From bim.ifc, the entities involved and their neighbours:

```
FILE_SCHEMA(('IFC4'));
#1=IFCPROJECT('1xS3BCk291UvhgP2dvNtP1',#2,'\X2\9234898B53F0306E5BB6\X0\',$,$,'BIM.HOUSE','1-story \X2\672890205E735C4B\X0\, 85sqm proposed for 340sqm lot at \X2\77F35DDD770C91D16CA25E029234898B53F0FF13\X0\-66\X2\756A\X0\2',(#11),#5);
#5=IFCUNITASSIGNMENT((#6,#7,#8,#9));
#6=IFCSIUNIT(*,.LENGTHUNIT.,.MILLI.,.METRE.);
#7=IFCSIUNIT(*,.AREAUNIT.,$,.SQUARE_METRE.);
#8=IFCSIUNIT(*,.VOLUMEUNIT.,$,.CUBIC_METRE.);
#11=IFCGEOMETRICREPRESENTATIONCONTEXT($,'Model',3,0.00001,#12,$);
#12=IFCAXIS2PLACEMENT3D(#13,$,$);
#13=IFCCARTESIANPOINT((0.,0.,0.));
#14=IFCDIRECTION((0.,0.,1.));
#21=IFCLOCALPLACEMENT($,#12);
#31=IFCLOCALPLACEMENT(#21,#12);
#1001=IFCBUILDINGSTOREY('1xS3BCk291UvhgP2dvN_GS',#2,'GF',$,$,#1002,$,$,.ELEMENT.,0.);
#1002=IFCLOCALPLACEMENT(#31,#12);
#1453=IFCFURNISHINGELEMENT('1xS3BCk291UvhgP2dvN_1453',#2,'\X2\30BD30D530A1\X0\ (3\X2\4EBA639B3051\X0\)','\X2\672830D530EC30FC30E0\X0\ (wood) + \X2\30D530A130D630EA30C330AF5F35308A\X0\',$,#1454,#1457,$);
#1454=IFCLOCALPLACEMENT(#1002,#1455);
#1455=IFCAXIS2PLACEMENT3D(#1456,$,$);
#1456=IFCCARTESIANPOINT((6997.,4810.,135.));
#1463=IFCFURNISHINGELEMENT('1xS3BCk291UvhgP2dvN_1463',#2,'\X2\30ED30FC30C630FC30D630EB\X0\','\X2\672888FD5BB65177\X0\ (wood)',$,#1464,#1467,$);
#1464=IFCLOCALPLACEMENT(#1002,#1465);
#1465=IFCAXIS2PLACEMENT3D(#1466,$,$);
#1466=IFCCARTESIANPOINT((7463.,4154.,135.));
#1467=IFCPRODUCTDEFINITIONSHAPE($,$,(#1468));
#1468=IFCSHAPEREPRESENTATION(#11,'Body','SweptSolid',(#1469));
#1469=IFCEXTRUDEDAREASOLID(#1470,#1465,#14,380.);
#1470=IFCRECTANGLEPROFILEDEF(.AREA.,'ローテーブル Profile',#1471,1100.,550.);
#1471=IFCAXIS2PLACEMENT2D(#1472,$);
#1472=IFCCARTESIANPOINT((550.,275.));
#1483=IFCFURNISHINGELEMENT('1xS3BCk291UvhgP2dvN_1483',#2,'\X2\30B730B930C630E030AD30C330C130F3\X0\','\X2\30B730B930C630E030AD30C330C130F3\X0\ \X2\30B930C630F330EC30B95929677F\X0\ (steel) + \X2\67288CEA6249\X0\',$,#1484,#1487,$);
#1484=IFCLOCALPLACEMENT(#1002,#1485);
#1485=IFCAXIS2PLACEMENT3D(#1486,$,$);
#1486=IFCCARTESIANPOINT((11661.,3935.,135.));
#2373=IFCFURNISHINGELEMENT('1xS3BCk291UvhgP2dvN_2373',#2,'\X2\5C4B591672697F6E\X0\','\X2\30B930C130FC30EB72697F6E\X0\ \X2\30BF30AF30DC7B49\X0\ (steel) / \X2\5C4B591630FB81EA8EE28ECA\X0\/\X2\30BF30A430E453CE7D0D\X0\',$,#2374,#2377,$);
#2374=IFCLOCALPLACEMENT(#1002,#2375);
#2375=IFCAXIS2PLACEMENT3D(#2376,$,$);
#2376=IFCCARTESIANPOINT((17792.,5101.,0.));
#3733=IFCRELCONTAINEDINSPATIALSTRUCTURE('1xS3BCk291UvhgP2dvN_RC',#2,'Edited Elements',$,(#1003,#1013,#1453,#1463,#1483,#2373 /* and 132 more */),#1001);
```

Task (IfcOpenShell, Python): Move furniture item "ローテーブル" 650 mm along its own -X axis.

```python
import ifcopenshell
import ifcopenshell.api.geometry
import ifcopenshell.util.placement
import ifcopenshell.util.unit

model = ifcopenshell.open("bim.ifc")
unit_scale = ifcopenshell.util.unit.calculate_unit_scale(model)

item = model.by_guid("1xS3BCk291UvhgP2dvN_1463")
matrix = ifcopenshell.util.placement.get_local_placement(item.ObjectPlacement)
matrix[:3, 3] -= matrix[:3, 0] * 0.65 / unit_scale
ifcopenshell.api.geometry.edit_object_placement(model, product=item, matrix=matrix, is_si=False)

print(ifcopenshell.util.placement.get_local_placement(item.ObjectPlacement).round(3) + 0.0)

model.write("bim_updated.ifc")
```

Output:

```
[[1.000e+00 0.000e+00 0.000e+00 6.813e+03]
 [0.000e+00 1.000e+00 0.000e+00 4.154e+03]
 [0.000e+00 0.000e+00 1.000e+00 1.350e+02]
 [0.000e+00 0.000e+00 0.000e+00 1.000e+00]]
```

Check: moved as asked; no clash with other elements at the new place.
